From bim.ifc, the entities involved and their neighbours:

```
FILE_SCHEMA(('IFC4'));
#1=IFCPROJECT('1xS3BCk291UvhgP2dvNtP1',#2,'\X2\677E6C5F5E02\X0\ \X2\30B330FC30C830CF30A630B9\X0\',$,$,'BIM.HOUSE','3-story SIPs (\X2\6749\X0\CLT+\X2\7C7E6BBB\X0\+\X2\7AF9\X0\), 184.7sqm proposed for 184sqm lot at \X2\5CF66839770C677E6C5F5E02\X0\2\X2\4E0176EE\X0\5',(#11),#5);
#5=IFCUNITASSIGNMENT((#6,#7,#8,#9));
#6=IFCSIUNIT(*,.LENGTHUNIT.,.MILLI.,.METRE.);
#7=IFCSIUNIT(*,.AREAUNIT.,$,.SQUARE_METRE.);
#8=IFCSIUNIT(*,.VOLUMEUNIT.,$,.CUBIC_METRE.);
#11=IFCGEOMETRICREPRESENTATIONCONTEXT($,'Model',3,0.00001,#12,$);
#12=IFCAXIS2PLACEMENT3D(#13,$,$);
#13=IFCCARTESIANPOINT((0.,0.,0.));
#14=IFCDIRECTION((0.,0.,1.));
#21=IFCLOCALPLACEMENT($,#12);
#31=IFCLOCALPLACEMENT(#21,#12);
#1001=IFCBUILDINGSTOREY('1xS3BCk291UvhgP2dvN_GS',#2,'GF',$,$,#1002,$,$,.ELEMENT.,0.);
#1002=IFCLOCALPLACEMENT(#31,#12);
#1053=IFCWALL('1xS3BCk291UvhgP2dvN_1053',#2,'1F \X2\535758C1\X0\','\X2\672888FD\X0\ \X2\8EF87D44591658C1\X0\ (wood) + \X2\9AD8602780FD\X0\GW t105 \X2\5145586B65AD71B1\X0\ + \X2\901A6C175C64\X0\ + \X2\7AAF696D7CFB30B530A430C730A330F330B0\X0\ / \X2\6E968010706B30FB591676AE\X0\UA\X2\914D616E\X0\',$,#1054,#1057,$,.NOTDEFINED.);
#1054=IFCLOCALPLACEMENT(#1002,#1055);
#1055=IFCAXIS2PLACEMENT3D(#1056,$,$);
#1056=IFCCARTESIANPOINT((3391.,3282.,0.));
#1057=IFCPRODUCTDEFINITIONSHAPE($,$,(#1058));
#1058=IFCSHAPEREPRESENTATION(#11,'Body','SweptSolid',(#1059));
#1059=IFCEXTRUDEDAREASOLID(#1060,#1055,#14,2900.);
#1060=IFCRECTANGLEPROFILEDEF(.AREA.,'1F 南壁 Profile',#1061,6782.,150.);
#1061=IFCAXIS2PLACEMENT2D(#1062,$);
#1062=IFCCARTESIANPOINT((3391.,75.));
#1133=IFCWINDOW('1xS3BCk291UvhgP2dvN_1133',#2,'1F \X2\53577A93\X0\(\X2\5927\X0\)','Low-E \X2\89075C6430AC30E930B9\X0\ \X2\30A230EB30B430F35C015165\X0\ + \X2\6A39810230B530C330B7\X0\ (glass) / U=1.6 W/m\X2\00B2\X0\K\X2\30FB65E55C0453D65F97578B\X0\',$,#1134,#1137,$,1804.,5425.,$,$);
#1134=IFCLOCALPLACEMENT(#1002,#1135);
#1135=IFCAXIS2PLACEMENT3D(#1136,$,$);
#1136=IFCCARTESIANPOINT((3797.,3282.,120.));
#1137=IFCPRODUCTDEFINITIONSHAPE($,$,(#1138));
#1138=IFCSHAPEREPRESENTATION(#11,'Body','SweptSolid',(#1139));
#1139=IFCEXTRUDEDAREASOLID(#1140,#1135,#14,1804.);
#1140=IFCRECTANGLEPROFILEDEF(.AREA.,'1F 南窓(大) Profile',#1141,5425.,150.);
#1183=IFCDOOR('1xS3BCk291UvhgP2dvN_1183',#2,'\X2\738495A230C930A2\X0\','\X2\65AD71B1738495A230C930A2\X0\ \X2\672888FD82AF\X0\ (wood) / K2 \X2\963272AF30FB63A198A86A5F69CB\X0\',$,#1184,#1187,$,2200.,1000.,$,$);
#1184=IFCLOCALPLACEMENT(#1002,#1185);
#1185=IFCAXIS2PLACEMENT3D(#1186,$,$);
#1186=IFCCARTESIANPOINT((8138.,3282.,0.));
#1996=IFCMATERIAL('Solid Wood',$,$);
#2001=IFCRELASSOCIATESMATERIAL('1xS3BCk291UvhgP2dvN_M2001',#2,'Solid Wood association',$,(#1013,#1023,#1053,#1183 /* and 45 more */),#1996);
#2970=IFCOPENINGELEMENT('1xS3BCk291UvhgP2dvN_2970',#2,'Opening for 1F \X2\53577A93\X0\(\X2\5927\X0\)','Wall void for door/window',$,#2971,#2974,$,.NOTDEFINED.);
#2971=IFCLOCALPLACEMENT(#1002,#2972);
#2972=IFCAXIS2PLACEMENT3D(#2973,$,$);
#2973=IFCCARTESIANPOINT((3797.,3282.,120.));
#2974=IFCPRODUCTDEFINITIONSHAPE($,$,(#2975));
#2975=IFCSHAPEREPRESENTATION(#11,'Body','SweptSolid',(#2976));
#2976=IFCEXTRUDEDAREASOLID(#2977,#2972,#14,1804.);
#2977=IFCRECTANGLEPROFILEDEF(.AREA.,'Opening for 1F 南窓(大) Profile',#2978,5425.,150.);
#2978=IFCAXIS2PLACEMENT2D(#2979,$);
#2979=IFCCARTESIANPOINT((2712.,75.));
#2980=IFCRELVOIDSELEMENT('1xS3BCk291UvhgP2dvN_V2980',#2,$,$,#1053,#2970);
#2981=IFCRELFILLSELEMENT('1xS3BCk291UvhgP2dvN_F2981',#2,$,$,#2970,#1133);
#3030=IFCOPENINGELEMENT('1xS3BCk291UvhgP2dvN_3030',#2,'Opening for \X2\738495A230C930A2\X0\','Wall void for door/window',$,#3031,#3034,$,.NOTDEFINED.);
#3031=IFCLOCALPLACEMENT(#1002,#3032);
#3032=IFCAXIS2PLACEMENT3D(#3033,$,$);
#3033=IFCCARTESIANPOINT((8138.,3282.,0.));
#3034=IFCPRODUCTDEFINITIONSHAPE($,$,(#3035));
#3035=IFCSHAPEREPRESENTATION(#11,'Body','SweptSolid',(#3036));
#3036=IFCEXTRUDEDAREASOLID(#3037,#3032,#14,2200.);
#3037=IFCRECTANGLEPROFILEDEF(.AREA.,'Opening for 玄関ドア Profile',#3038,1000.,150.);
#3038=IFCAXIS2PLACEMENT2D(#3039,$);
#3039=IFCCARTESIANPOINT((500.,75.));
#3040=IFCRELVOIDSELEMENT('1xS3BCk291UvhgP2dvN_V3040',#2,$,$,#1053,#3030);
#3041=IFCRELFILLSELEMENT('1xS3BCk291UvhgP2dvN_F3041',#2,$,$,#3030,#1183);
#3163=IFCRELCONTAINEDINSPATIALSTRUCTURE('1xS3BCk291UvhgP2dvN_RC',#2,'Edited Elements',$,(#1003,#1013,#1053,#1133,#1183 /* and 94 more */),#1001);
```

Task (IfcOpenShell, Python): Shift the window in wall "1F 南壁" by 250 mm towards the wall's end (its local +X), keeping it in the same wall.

```python
import ifcopenshell
import ifcopenshell.api.geometry
import ifcopenshell.util.placement
import ifcopenshell.util.unit

model = ifcopenshell.open("bim.ifc")
unit_scale = ifcopenshell.util.unit.calculate_unit_scale(model)

window = model.by_guid("1xS3BCk291UvhgP2dvN_1133")
opening = window.FillsVoids[0].RelatingOpeningElement
wall = opening.VoidsElements[0].RelatingBuildingElement

wall_matrix = ifcopenshell.util.placement.get_local_placement(wall.ObjectPlacement)
shift = wall_matrix[:3, 0] * 0.25 / unit_scale
before = ifcopenshell.util.placement.get_local_placement(window.ObjectPlacement)[:3, 3].copy()

# The window is not placed relative to its opening, so move both.
for product in (opening, window):
    matrix = ifcopenshell.util.placement.get_local_placement(product.ObjectPlacement)
    matrix[:3, 3] += shift
    ifcopenshell.api.geometry.edit_object_placement(model, product=product, matrix=matrix, is_si=False)

after = ifcopenshell.util.placement.get_local_placement(window.ObjectPlacement)[:3, 3]
print("window moved by", (after - before).round(3) + 0.0)

model.write("bim_updated.ifc")
```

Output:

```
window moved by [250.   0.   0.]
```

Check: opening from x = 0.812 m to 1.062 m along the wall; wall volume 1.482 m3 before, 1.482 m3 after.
